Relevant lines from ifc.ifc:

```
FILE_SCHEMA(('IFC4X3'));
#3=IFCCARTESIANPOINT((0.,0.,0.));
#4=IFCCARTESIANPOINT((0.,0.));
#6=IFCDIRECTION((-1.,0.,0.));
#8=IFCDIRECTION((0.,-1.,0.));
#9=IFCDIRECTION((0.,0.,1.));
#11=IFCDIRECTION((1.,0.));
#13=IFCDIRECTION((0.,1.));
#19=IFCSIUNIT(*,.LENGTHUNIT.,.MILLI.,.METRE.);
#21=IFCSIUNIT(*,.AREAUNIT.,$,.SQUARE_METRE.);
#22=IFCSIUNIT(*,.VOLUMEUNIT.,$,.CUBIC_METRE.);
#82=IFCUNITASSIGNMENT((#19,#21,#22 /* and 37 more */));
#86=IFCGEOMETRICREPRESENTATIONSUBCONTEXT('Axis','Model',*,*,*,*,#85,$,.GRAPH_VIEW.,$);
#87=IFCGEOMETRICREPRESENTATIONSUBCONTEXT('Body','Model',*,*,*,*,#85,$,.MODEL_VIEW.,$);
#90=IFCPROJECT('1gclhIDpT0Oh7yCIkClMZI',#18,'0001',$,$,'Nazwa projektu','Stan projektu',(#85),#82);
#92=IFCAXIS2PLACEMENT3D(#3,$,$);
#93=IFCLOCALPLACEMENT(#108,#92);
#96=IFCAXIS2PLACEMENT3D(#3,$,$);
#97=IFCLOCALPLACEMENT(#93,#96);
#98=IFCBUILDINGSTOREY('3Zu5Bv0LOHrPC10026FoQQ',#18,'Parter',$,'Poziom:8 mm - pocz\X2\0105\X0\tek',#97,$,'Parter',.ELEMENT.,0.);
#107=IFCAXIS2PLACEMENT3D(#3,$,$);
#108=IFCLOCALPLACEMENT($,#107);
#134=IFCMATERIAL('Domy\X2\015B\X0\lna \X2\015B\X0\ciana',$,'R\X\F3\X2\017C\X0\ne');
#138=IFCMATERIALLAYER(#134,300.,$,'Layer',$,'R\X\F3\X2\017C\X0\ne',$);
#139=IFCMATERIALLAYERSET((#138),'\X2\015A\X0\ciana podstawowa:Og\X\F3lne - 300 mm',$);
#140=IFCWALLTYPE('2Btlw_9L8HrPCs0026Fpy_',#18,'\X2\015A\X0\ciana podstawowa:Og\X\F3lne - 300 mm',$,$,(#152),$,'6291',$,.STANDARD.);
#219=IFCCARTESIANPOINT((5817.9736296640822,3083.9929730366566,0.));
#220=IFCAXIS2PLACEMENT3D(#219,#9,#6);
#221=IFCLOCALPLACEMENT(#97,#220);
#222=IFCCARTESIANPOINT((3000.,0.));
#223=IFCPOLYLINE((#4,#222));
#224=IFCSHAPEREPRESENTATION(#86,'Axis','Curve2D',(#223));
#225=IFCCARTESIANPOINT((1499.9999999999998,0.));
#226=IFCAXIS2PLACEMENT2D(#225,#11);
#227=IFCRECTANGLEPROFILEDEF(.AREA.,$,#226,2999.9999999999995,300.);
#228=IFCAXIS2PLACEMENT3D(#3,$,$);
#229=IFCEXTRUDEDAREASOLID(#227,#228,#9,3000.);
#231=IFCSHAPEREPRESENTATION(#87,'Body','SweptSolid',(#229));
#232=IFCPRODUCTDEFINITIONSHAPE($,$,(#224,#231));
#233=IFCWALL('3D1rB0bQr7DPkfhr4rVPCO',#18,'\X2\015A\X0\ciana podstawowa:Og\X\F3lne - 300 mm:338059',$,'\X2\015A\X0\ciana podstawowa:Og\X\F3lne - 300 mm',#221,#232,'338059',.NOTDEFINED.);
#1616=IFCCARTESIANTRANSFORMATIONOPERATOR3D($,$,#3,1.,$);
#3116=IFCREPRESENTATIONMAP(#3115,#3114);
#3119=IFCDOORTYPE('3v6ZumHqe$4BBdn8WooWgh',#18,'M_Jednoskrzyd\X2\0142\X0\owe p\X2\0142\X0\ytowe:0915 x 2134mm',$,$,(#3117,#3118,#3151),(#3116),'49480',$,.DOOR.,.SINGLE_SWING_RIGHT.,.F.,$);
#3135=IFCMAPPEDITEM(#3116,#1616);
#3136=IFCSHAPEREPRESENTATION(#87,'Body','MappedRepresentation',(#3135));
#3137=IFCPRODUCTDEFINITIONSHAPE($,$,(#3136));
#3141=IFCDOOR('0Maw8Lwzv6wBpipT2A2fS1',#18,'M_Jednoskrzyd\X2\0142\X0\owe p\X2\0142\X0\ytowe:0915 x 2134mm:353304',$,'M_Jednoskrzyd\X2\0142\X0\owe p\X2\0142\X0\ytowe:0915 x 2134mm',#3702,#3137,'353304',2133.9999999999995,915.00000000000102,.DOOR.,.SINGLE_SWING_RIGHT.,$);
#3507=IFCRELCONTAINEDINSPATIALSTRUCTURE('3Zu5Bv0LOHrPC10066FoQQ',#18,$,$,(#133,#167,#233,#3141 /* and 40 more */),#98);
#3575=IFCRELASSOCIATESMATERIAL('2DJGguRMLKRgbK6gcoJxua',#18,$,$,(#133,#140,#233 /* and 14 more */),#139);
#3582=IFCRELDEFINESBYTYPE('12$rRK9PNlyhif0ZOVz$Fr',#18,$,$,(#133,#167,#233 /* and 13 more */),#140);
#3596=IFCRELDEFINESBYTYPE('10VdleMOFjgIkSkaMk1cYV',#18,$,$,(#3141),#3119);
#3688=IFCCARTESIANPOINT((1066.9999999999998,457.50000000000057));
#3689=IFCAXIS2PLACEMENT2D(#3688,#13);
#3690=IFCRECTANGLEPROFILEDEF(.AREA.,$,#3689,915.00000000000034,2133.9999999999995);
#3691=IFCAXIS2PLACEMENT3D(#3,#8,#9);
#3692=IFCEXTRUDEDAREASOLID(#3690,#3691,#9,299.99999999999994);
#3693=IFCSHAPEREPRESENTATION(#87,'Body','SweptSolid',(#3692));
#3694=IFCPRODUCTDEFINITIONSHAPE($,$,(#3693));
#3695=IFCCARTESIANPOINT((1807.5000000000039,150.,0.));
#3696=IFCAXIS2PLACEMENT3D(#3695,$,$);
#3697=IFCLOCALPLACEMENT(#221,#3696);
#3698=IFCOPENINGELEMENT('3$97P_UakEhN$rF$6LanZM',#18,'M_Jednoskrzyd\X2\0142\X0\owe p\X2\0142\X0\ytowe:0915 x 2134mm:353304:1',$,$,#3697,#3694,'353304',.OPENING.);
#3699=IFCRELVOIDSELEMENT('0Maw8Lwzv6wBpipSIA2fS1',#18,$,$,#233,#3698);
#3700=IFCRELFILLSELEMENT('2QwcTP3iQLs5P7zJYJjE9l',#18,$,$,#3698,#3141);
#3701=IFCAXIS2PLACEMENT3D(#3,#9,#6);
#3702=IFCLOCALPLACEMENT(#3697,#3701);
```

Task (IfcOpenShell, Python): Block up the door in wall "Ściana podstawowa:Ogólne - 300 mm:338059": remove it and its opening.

```python
import ifcopenshell
import ifcopenshell.api.feature
import ifcopenshell.api.root
import ifcopenshell.geom
import ifcopenshell.util.shape

model = ifcopenshell.open("ifc.ifc")
settings = ifcopenshell.geom.settings()


def volume(element):
    """Net volume in cubic metres, openings subtracted."""
    shape = ifcopenshell.geom.create_shape(settings, element)
    return ifcopenshell.util.shape.get_volume(shape.geometry)


door = model.by_guid("0Maw8Lwzv6wBpipT2A2fS1")
opening = door.FillsVoids[0].RelatingOpeningElement
wall = opening.VoidsElements[0].RelatingBuildingElement
before = volume(wall)

ifcopenshell.api.root.remove_product(model, product=door)
ifcopenshell.api.feature.remove_feature(model, feature=opening)

after = volume(wall)

print(f"wall volume {before:.3f} -> {after:.3f} m3")

model.write("ifc_edited.ifc")
```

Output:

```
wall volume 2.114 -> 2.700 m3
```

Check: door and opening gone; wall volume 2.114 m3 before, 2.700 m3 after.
